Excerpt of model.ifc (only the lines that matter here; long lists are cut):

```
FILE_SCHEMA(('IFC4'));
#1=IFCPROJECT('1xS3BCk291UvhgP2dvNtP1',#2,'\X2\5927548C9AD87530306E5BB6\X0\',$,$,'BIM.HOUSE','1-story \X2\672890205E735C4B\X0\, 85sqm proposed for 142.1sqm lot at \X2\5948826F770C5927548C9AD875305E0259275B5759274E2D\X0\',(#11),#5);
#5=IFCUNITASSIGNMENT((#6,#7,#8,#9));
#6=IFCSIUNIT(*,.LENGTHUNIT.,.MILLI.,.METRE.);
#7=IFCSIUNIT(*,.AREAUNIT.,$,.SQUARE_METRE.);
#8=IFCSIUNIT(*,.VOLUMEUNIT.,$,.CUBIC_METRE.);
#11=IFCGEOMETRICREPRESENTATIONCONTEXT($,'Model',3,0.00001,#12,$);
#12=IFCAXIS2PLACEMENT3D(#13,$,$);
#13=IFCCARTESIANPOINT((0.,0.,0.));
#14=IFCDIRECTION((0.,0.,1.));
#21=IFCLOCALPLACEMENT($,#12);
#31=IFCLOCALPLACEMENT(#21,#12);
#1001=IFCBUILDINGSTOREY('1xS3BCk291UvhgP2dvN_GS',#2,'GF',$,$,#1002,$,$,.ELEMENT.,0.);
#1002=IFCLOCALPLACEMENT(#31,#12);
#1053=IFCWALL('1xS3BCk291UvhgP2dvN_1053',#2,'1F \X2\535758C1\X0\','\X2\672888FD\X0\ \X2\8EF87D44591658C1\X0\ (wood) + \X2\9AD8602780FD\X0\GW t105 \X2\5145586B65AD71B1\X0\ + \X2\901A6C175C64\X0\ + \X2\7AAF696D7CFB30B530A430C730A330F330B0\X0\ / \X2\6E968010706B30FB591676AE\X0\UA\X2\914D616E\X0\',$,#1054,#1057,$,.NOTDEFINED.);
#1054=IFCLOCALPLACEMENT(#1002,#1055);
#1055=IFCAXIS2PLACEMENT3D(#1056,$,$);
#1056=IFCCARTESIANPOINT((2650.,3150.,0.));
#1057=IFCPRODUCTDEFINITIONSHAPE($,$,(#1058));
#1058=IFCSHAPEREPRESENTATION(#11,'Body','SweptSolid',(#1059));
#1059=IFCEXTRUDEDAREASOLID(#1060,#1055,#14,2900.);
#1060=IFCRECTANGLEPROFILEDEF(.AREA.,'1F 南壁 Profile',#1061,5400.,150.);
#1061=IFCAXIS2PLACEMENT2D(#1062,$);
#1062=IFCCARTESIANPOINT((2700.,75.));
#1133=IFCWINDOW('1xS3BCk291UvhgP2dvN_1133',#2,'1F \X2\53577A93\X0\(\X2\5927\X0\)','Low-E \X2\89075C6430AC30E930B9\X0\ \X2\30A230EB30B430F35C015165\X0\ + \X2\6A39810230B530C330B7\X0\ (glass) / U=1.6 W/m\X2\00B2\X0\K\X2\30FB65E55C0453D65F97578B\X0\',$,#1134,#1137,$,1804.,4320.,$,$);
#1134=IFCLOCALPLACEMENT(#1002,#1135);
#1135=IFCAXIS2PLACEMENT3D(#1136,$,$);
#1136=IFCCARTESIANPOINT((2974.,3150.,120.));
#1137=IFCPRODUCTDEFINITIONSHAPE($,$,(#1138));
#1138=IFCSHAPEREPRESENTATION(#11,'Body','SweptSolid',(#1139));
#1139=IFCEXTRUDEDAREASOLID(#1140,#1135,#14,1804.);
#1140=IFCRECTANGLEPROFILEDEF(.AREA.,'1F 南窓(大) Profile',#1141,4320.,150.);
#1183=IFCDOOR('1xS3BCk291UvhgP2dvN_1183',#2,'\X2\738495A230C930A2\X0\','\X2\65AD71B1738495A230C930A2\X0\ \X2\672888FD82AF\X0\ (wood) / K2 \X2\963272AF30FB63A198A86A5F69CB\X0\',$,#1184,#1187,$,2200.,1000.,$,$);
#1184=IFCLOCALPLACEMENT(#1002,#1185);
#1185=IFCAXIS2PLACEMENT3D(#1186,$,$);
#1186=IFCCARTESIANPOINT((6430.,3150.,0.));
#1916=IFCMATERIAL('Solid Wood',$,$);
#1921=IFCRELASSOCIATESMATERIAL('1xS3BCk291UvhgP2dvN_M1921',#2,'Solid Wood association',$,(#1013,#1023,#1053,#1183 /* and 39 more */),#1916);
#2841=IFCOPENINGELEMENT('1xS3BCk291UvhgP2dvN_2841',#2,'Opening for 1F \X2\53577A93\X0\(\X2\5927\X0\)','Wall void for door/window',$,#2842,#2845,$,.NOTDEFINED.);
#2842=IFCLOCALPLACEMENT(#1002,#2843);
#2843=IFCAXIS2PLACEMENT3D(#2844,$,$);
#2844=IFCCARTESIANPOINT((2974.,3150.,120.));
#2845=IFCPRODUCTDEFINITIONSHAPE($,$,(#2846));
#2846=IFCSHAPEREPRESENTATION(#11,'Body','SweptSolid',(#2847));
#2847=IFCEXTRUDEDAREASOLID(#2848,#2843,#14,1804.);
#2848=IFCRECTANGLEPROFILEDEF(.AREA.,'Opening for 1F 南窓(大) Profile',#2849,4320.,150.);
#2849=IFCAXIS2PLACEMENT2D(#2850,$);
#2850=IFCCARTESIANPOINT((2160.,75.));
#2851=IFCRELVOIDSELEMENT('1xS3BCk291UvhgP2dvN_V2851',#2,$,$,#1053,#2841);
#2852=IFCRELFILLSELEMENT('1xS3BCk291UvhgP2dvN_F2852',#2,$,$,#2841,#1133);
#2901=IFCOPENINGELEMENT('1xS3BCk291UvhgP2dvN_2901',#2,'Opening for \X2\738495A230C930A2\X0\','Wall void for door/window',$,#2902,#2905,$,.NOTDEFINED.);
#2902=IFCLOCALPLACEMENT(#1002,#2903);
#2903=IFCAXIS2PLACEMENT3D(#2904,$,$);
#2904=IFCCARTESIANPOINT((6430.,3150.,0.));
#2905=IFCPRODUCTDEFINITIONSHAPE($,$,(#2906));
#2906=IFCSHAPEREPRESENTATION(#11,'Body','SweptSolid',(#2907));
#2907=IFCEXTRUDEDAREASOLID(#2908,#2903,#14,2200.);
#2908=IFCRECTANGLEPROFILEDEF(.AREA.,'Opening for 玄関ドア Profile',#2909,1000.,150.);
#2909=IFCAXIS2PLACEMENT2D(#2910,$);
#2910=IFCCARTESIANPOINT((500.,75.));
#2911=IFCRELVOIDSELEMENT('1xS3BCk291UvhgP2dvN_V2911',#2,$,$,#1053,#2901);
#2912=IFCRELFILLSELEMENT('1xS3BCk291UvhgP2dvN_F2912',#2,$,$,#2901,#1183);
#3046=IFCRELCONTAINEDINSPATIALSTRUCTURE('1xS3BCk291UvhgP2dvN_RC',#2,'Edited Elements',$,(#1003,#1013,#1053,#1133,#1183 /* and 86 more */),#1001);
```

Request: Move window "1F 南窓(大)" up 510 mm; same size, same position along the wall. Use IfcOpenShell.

```python
import numpy as np
import ifcopenshell
import ifcopenshell.api.geometry
import ifcopenshell.util.placement
import ifcopenshell.util.unit

model = ifcopenshell.open("model.ifc")
unit_scale = ifcopenshell.util.unit.calculate_unit_scale(model)

window = model.by_id(1133)
opening = window.FillsVoids[0].RelatingOpeningElement
dz = 510.0

shift = np.array([0.0, 0.0, dz])
# The window is not placed relative to its opening, so move both.
for product in (opening, window):
    matrix = ifcopenshell.util.placement.get_local_placement(product.ObjectPlacement)
    matrix[:3, 3] += shift
    ifcopenshell.api.geometry.edit_object_placement(model, product=product, matrix=matrix, is_si=False)

print(f"moved by {dz * unit_scale:+.3f} m")

model.write("model_v2.ifc")
```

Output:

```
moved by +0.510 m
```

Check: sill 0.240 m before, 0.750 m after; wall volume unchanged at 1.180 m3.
